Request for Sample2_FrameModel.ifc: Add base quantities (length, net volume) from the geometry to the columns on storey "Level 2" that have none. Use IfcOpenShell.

First a look at what the model holds.

```python
import ifcopenshell
import ifcopenshell.util.element
import ifcopenshell.util.unit

model = ifcopenshell.open("Sample2_FrameModel.ifc")
print(model.schema)
for unit_type in ("LENGTHUNIT", "AREAUNIT", "VOLUMEUNIT"):
    print(unit_type, ifcopenshell.util.unit.calculate_unit_scale(model, unit_type))
storey = next(s for s in model.by_type("IfcBuildingStorey") if s.Name == "Level 2")
columns = [e for e in ifcopenshell.util.element.get_decomposition(storey) if e.is_a("IfcColumn")]
for e in sorted(columns, key=lambda e: e.id()):
    print(e.id(), e.is_a(), e.Name, list(ifcopenshell.util.element.get_psets(e, qtos_only=True)), sep=" | ")
```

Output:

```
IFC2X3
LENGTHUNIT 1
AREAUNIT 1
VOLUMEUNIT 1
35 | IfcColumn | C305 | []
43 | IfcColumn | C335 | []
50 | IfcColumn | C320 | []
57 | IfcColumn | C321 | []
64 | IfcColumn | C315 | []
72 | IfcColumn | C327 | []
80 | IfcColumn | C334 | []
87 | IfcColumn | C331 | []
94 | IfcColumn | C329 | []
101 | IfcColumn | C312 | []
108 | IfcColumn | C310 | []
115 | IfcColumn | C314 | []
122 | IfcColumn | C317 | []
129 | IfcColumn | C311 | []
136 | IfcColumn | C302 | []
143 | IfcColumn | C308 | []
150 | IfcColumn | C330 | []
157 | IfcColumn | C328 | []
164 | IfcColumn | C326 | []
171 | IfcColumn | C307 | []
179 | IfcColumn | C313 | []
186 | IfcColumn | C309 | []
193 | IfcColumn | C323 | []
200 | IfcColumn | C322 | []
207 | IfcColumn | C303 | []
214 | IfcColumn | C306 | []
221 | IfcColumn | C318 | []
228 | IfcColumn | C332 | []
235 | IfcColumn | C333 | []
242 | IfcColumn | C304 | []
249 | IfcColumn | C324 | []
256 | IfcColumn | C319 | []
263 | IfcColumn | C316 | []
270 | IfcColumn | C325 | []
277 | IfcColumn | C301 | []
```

```python
import ifcopenshell
import ifcopenshell.api.pset
import ifcopenshell.geom
import ifcopenshell.util.element
import ifcopenshell.util.shape
import ifcopenshell.util.unit

model = ifcopenshell.open("Sample2_FrameModel.ifc")
unit_scale = ifcopenshell.util.unit.calculate_unit_scale(model)
volume_scale = ifcopenshell.util.unit.calculate_unit_scale(model, "VOLUMEUNIT")
settings = ifcopenshell.geom.settings()

storey = next(s for s in model.by_type("IfcBuildingStorey") if s.Name == "Level 2")
columns = [e for e in ifcopenshell.util.element.get_decomposition(storey) if e.is_a("IfcColumn")]

for e in sorted(columns, key=lambda e: e.id()):
    if ifcopenshell.util.element.get_psets(e, qtos_only=True, should_inherit=False):
        continue
    # Geometry comes back in metres, in the element's own axes.
    shape = ifcopenshell.geom.create_shape(settings, e)
    values = {
        "Length": ifcopenshell.util.shape.get_z(shape.geometry) / unit_scale,
        "NetVolume": ifcopenshell.util.shape.get_volume(shape.geometry) / volume_scale,
    }
    qto = ifcopenshell.api.pset.add_qto(model, product=e, name="BaseQuantities")
    ifcopenshell.api.pset.edit_qto(model, qto=qto, properties=values)
    print(e.id(), {k: round(v, 3) for k, v in values.items()})

model.write("Sample2_FrameModel_updated.ifc")
```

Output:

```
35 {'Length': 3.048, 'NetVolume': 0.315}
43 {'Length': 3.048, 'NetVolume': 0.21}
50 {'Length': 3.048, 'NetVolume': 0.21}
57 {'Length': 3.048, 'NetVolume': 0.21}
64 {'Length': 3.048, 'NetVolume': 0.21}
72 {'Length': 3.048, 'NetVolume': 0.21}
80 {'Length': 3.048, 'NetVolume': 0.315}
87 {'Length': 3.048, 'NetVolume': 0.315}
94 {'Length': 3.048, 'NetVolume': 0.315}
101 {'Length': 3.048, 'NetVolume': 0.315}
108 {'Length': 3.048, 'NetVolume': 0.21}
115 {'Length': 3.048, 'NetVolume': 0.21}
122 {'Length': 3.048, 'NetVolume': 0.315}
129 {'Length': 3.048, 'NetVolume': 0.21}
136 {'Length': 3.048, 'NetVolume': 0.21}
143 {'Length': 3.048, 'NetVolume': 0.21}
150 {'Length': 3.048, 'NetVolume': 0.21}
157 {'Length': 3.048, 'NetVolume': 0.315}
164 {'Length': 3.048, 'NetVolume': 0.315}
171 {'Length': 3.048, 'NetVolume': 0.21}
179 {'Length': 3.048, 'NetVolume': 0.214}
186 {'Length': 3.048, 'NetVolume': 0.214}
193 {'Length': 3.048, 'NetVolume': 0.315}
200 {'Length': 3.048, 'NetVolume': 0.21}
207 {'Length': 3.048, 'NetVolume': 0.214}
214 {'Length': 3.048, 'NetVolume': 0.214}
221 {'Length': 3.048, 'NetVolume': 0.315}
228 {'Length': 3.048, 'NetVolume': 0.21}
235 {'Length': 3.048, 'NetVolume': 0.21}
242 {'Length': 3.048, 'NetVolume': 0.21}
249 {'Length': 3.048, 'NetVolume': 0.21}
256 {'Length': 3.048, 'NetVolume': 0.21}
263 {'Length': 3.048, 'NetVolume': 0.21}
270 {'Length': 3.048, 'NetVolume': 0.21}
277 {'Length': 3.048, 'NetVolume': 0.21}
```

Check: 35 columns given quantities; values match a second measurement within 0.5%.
